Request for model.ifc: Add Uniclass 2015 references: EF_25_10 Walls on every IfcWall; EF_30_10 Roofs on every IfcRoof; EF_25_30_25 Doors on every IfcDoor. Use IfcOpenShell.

First a look at what the model holds.

```python
import ifcopenshell

model = ifcopenshell.open("model.ifc")
print(model.schema)
print("classifications:", [c.Name for c in model.by_type("IfcClassification")])
for ifc_class in ("IfcDoor", "IfcRoof", "IfcStair", "IfcWall", "IfcWindow"):
    print(ifc_class, len(model.by_type(ifc_class)))
```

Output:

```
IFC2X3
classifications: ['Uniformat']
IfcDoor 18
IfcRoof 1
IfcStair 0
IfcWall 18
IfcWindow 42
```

```python
import ifcopenshell
import ifcopenshell.api.classification

model = ifcopenshell.open("model.ifc")

# IFC2X3 requires Source and Edition and has no link from the project to the system.
system = model.create_entity("IfcClassification", Source="NBS", Edition="2015", Name="Uniclass 2015")

codes = {
    "IfcWall": ("EF_25_10", "Walls"),
    "IfcRoof": ("EF_30_10", "Roofs"),
    "IfcDoor": ("EF_25_30_25", "Doors"),
}
for ifc_class, (code, name) in codes.items():
    products = model.by_type(ifc_class)
    ifcopenshell.api.classification.add_reference(
        model, products=products, classification=system, identification=code, name=name
    )
    print(code, len(products))

model.write("model_edited.ifc")
```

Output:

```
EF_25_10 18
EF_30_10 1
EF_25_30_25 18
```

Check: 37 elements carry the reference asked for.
